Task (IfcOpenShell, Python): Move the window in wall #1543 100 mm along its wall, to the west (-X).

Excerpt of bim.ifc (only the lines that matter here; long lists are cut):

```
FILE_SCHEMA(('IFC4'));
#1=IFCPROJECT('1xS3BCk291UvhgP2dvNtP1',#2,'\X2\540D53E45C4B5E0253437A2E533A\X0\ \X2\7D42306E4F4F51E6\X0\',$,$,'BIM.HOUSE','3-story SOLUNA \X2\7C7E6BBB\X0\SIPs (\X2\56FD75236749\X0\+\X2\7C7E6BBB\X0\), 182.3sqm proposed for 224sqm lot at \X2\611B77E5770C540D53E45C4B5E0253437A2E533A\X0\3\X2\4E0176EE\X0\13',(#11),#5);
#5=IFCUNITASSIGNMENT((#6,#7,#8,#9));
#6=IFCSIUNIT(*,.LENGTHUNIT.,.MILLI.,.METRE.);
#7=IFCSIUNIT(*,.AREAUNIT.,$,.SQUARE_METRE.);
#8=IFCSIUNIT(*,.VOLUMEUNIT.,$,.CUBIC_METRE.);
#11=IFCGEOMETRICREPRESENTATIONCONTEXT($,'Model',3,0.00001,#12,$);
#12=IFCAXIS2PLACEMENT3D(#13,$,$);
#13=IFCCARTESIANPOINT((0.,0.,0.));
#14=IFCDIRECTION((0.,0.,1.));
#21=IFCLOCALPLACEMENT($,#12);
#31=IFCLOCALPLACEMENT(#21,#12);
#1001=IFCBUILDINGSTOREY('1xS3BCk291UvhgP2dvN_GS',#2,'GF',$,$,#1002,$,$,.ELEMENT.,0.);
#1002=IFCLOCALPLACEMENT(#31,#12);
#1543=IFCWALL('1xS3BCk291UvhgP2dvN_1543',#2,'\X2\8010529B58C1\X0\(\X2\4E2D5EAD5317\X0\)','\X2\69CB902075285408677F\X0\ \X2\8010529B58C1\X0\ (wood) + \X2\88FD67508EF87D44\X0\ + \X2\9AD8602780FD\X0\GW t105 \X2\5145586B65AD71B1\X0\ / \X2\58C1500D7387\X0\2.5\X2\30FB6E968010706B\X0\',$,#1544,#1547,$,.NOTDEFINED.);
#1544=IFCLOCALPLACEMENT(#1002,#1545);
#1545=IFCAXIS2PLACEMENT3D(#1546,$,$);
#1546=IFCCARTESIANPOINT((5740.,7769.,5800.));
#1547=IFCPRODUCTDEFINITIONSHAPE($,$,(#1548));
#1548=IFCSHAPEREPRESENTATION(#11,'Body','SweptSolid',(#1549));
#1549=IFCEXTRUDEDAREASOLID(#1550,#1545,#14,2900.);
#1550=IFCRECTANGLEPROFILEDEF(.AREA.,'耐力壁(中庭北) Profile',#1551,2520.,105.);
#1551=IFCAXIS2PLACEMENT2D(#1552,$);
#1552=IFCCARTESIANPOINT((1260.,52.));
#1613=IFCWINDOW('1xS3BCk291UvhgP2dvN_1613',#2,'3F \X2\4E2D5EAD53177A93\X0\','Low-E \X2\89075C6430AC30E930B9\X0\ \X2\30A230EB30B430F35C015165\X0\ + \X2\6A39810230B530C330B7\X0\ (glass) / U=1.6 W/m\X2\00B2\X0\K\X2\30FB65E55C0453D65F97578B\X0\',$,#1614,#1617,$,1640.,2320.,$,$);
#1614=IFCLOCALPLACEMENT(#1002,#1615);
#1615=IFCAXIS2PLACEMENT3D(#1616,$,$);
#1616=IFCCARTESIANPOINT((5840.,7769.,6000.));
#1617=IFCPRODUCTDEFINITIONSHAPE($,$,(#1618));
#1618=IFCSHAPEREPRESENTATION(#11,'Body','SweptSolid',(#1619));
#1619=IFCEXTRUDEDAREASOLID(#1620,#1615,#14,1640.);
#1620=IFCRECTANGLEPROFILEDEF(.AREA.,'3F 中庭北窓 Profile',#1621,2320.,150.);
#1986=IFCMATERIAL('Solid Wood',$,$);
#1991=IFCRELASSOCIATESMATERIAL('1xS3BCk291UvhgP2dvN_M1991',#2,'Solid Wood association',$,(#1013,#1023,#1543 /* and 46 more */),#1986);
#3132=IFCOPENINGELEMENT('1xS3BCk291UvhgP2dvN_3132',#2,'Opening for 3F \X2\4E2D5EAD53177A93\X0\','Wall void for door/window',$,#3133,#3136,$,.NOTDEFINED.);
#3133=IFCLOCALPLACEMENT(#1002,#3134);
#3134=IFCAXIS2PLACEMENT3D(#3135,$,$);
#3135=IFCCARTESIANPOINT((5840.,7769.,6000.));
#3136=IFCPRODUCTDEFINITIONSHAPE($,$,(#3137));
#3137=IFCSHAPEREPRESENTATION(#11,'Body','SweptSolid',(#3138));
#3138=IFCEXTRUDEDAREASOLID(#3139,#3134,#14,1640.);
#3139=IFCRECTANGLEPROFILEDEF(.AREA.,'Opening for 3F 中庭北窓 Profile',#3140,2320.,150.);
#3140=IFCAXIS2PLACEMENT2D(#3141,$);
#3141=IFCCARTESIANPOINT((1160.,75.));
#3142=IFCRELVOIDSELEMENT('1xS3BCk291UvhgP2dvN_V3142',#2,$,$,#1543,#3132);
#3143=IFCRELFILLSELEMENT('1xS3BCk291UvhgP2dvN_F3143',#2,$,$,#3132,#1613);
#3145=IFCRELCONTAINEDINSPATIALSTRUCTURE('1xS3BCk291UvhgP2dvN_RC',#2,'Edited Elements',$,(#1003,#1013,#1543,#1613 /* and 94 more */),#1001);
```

```python
import ifcopenshell
import ifcopenshell.api.geometry
import ifcopenshell.util.placement
import ifcopenshell.util.unit

model = ifcopenshell.open("bim.ifc")
unit_scale = ifcopenshell.util.unit.calculate_unit_scale(model)

window = model.by_id(1613)
opening = window.FillsVoids[0].RelatingOpeningElement
wall = opening.VoidsElements[0].RelatingBuildingElement

wall_matrix = ifcopenshell.util.placement.get_local_placement(wall.ObjectPlacement)
shift = wall_matrix[:3, 0] * -0.1 / unit_scale
before = ifcopenshell.util.placement.get_local_placement(window.ObjectPlacement)[:3, 3].copy()

# The window is not placed relative to its opening, so move both.
for product in (opening, window):
    matrix = ifcopenshell.util.placement.get_local_placement(product.ObjectPlacement)
    matrix[:3, 3] += shift
    ifcopenshell.api.geometry.edit_object_placement(model, product=product, matrix=matrix, is_si=False)

after = ifcopenshell.util.placement.get_local_placement(window.ObjectPlacement)[:3, 3]
print("window moved by", (after - before).round(3) + 0.0)

model.write("bim_edited.ifc")
```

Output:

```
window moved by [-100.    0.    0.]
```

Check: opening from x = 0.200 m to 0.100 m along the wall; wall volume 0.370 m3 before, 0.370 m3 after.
